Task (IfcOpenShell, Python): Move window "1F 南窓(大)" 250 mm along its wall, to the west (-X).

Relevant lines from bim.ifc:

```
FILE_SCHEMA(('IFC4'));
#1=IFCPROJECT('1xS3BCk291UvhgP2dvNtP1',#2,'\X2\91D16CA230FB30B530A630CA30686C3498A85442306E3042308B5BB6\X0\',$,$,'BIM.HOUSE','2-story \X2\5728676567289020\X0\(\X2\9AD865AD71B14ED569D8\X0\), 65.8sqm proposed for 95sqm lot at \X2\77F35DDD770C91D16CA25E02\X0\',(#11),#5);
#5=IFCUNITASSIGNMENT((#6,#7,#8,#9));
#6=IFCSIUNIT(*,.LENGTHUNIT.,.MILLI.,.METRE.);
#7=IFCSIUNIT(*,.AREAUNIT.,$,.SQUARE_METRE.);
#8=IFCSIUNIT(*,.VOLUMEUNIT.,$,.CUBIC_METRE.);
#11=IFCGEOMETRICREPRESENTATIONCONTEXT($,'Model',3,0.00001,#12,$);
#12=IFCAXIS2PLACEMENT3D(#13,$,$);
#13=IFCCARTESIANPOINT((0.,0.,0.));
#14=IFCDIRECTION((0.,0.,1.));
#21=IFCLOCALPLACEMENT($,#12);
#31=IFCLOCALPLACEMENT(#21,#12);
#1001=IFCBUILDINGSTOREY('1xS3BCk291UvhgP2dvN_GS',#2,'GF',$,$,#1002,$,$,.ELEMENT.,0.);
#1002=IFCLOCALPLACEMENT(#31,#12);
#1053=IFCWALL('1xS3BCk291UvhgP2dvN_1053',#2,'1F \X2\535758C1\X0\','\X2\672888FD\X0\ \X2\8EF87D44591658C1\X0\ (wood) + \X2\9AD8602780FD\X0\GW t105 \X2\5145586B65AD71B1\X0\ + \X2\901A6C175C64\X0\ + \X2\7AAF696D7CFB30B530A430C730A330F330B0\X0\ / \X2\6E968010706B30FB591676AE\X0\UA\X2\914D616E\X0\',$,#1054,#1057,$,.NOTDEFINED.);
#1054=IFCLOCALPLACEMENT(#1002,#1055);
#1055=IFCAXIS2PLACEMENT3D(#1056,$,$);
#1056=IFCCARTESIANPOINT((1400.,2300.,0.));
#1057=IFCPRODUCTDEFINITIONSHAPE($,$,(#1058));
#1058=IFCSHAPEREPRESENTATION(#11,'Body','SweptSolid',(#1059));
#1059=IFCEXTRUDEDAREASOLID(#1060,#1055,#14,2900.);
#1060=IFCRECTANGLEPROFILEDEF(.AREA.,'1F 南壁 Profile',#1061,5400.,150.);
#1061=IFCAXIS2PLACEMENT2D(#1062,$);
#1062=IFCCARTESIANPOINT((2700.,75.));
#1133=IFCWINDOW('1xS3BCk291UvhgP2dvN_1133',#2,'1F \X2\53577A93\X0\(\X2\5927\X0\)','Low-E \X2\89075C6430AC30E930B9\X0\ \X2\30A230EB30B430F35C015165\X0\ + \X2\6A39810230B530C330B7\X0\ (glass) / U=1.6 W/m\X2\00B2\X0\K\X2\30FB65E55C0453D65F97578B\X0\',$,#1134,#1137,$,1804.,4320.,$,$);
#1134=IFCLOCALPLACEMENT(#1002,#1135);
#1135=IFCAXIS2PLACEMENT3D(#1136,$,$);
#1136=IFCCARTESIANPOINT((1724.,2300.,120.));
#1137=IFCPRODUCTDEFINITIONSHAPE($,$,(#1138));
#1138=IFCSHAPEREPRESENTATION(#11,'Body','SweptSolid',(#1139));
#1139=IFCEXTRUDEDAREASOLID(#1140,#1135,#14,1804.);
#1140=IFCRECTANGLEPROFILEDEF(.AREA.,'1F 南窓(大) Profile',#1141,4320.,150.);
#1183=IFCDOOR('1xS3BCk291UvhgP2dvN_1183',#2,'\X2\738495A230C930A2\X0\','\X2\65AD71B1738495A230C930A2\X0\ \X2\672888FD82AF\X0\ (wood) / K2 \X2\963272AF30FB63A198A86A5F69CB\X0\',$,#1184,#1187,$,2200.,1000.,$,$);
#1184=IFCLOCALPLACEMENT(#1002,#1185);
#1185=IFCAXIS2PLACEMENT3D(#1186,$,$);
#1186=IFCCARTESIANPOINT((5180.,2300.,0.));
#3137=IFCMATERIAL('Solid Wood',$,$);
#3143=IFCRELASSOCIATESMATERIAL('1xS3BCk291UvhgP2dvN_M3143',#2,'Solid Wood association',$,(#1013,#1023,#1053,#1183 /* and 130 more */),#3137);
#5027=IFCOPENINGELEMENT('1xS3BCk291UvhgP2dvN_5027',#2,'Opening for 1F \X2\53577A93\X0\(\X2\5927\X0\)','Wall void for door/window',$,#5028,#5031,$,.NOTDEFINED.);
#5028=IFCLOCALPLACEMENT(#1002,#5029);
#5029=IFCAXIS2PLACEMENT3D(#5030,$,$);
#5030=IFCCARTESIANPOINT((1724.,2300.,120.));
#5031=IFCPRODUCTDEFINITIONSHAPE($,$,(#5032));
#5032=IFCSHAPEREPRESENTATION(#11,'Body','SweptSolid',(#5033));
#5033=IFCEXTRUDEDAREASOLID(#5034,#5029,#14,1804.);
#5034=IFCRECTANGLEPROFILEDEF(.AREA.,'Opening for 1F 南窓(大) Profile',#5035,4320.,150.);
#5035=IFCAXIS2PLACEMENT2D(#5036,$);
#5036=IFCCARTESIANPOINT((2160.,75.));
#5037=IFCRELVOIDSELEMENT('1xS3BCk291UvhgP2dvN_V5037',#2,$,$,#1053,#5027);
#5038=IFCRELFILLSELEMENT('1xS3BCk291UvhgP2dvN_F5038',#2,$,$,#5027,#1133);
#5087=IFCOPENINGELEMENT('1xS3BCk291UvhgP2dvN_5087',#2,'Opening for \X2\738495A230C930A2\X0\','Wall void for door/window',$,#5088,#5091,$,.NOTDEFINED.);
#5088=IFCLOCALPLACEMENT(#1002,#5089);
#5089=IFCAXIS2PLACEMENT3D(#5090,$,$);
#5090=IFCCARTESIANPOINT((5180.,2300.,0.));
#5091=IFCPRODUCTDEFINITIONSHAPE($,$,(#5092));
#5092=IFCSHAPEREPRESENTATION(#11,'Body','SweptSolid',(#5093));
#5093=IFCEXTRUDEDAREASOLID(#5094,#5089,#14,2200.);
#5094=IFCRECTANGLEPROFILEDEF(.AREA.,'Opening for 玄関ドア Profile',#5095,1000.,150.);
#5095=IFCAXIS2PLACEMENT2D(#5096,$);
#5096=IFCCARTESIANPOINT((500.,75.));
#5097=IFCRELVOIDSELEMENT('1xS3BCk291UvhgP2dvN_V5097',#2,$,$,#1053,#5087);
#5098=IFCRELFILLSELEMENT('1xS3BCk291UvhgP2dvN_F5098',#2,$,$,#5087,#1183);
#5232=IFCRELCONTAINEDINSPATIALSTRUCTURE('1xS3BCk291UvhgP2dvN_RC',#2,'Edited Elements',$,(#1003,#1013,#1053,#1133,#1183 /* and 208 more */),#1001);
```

```python
import ifcopenshell
import ifcopenshell.api.geometry
import ifcopenshell.util.placement
import ifcopenshell.util.unit

model = ifcopenshell.open("bim.ifc")
unit_scale = ifcopenshell.util.unit.calculate_unit_scale(model)

window = model.by_id(1133)
opening = window.FillsVoids[0].RelatingOpeningElement
wall = opening.VoidsElements[0].RelatingBuildingElement

wall_matrix = ifcopenshell.util.placement.get_local_placement(wall.ObjectPlacement)
shift = wall_matrix[:3, 0] * -0.25 / unit_scale
before = ifcopenshell.util.placement.get_local_placement(window.ObjectPlacement)[:3, 3].copy()

# The window is not placed relative to its opening, so move both.
for product in (opening, window):
    matrix = ifcopenshell.util.placement.get_local_placement(product.ObjectPlacement)
    matrix[:3, 3] += shift
    ifcopenshell.api.geometry.edit_object_placement(model, product=product, matrix=matrix, is_si=False)

after = ifcopenshell.util.placement.get_local_placement(window.ObjectPlacement)[:3, 3]
print("window moved by", (after - before).round(3) + 0.0)

model.write("bim-out.ifc")
```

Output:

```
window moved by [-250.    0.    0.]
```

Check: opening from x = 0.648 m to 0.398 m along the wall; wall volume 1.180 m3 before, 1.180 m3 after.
